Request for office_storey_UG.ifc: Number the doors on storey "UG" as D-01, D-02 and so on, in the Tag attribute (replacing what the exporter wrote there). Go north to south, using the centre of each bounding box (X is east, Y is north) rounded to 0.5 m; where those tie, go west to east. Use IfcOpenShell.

First a look at what the model holds.

```python
import ifcopenshell
import ifcopenshell.util.element
import ifcopenshell.util.placement

model = ifcopenshell.open("office_storey_UG.ifc")
print(model.schema)
storey = next(s for s in model.by_type("IfcBuildingStorey") if s.Name == "UG")
doors = [e for e in ifcopenshell.util.element.get_decomposition(storey) if e.is_a("IfcDoor")]
for e in sorted(doors, key=lambda e: e.id()):
    origin = ifcopenshell.util.placement.get_local_placement(e.ObjectPlacement)[:3, 3]
    print(e.id(), e.Tag, e.Name, origin.round(2) + 0.0, sep=" | ")
```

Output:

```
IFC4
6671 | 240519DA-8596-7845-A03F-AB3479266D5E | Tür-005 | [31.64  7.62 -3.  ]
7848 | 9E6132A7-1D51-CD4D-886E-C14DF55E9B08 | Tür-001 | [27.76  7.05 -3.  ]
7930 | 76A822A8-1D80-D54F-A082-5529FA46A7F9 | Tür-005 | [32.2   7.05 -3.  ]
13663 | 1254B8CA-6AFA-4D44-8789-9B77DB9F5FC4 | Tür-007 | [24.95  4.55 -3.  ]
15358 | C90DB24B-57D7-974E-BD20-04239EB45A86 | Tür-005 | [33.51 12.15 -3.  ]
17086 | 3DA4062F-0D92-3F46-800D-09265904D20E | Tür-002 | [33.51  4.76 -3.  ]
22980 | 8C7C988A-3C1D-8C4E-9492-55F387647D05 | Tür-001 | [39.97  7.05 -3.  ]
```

```python
import ifcopenshell
import ifcopenshell.geom
import ifcopenshell.util.element
import ifcopenshell.util.shape

model = ifcopenshell.open("office_storey_UG.ifc")
settings = ifcopenshell.geom.settings()
settings.set("use-world-coords", True)


def centre(element):
    shape = ifcopenshell.geom.create_shape(settings, element)
    return ifcopenshell.util.shape.get_bbox_centroid(shape.geometry)


storey = next(s for s in model.by_type("IfcBuildingStorey") if s.Name == "UG")
doors = [e for e in ifcopenshell.util.element.get_decomposition(storey) if e.is_a("IfcDoor")]

# Insertion points can sit at a corner or the storey origin, so sort by the geometry (in metres).
centres = {e: centre(e) for e in doors}
doors.sort(key=lambda e: (-round(centres[e][1] / 0.5), centres[e][0]))

for i, e in enumerate(doors, start=1):
    number = f"D-{i:02d}"
    e.Tag = number
    print(e.id(), number)

model.write("office_storey_UG_v2.ifc")
```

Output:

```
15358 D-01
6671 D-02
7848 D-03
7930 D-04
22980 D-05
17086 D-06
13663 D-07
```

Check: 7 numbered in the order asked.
